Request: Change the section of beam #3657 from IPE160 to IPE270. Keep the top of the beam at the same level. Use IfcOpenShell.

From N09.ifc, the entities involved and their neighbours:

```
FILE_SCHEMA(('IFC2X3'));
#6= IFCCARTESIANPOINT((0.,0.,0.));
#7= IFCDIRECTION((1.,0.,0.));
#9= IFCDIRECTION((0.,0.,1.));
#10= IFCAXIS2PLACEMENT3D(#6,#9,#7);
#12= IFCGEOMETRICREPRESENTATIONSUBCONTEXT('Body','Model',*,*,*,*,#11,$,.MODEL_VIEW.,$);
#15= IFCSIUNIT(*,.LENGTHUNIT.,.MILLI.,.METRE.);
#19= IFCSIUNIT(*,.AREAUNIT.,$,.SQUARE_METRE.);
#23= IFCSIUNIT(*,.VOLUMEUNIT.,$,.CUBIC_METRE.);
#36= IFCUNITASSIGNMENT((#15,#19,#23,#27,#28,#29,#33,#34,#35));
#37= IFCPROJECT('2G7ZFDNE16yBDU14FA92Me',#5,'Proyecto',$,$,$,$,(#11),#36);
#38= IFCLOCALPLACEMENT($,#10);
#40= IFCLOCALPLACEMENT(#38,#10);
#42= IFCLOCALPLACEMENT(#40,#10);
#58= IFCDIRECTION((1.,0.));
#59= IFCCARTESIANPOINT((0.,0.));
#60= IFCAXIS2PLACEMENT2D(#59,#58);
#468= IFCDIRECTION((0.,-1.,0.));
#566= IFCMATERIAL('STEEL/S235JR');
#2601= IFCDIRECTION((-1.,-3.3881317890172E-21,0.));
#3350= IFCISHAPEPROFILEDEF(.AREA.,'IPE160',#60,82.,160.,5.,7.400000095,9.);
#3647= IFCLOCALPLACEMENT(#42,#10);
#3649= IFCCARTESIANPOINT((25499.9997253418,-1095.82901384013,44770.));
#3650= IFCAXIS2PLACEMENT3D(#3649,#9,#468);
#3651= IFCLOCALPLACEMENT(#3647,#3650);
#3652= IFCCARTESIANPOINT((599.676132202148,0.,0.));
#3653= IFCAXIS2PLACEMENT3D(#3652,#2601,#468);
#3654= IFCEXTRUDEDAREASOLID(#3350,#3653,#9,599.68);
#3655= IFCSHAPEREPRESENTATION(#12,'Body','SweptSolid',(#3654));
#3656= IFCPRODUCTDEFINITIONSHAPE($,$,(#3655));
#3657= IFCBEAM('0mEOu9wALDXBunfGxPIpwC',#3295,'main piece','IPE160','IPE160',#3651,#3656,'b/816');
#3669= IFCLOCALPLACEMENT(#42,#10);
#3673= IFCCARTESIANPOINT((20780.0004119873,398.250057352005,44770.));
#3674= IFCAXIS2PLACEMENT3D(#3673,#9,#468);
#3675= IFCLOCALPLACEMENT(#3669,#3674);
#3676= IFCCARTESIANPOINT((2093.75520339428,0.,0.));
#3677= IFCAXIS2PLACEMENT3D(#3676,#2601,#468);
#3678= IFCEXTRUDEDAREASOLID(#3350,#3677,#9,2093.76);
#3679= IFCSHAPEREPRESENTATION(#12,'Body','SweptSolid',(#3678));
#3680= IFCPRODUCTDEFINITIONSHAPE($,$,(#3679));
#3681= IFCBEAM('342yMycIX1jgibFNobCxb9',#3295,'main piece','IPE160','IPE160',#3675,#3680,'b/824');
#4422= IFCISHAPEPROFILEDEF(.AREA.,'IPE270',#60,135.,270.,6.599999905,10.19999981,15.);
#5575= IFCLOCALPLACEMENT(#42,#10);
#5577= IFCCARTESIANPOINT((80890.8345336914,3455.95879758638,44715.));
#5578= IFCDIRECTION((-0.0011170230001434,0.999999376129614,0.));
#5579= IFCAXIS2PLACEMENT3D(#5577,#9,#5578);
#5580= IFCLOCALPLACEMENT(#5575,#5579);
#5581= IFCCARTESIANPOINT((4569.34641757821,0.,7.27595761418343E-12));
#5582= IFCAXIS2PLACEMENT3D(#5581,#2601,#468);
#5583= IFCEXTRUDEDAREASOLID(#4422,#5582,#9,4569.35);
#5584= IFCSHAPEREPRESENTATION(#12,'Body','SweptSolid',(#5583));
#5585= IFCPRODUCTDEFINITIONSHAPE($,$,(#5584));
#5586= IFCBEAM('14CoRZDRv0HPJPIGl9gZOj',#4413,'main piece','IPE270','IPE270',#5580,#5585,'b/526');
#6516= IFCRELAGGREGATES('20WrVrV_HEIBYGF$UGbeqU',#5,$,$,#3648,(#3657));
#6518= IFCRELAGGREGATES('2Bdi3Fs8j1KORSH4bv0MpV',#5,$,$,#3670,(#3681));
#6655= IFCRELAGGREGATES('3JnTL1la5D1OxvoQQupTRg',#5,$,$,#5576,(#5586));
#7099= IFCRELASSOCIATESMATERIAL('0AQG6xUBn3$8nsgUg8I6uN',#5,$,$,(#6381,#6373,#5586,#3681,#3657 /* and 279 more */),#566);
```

```python
import ifcopenshell
import ifcopenshell.util.element
import ifcopenshell.util.representation

model = ifcopenshell.open("N09.ifc")

member = model.by_guid("0mEOu9wALDXBunfGxPIpwC")
source = next(p for p in model.by_type("IfcIShapeProfileDef") if p.ProfileName == "IPE270")

body = ifcopenshell.util.representation.get_representation(member, "Model", "Body")
solid = body.Items[0]
old_profile = solid.SweptArea

# Copy the section's sizes but keep this member's own profile position.
profile = ifcopenshell.util.element.copy(model, source)
# Profiles are centred, so shift by half the change in depth to hold the top.
shift = (old_profile.OverallDepth - profile.OverallDepth) / 2
x, y = old_profile.Position.Location.Coordinates
up = (0.0, 1.0)  # upwards, in the solid's own plane
location = model.createIfcCartesianPoint((x + up[0] * shift, y + up[1] * shift))
profile.Position = model.createIfcAxis2Placement2D(location, old_profile.Position.RefDirection)
solid.SweptArea = profile
if not model.get_total_inverses(old_profile):
    ifcopenshell.util.element.remove_deep2(model, old_profile)
member.Description = member.Description.replace("IPE160", "IPE270")
member.ObjectType = member.ObjectType.replace("IPE160", "IPE270")

print(solid.SweptArea)

model.write("N09_v2.ifc")
```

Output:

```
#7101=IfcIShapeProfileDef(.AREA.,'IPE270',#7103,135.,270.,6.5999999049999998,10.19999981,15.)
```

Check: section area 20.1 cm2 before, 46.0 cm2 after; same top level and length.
